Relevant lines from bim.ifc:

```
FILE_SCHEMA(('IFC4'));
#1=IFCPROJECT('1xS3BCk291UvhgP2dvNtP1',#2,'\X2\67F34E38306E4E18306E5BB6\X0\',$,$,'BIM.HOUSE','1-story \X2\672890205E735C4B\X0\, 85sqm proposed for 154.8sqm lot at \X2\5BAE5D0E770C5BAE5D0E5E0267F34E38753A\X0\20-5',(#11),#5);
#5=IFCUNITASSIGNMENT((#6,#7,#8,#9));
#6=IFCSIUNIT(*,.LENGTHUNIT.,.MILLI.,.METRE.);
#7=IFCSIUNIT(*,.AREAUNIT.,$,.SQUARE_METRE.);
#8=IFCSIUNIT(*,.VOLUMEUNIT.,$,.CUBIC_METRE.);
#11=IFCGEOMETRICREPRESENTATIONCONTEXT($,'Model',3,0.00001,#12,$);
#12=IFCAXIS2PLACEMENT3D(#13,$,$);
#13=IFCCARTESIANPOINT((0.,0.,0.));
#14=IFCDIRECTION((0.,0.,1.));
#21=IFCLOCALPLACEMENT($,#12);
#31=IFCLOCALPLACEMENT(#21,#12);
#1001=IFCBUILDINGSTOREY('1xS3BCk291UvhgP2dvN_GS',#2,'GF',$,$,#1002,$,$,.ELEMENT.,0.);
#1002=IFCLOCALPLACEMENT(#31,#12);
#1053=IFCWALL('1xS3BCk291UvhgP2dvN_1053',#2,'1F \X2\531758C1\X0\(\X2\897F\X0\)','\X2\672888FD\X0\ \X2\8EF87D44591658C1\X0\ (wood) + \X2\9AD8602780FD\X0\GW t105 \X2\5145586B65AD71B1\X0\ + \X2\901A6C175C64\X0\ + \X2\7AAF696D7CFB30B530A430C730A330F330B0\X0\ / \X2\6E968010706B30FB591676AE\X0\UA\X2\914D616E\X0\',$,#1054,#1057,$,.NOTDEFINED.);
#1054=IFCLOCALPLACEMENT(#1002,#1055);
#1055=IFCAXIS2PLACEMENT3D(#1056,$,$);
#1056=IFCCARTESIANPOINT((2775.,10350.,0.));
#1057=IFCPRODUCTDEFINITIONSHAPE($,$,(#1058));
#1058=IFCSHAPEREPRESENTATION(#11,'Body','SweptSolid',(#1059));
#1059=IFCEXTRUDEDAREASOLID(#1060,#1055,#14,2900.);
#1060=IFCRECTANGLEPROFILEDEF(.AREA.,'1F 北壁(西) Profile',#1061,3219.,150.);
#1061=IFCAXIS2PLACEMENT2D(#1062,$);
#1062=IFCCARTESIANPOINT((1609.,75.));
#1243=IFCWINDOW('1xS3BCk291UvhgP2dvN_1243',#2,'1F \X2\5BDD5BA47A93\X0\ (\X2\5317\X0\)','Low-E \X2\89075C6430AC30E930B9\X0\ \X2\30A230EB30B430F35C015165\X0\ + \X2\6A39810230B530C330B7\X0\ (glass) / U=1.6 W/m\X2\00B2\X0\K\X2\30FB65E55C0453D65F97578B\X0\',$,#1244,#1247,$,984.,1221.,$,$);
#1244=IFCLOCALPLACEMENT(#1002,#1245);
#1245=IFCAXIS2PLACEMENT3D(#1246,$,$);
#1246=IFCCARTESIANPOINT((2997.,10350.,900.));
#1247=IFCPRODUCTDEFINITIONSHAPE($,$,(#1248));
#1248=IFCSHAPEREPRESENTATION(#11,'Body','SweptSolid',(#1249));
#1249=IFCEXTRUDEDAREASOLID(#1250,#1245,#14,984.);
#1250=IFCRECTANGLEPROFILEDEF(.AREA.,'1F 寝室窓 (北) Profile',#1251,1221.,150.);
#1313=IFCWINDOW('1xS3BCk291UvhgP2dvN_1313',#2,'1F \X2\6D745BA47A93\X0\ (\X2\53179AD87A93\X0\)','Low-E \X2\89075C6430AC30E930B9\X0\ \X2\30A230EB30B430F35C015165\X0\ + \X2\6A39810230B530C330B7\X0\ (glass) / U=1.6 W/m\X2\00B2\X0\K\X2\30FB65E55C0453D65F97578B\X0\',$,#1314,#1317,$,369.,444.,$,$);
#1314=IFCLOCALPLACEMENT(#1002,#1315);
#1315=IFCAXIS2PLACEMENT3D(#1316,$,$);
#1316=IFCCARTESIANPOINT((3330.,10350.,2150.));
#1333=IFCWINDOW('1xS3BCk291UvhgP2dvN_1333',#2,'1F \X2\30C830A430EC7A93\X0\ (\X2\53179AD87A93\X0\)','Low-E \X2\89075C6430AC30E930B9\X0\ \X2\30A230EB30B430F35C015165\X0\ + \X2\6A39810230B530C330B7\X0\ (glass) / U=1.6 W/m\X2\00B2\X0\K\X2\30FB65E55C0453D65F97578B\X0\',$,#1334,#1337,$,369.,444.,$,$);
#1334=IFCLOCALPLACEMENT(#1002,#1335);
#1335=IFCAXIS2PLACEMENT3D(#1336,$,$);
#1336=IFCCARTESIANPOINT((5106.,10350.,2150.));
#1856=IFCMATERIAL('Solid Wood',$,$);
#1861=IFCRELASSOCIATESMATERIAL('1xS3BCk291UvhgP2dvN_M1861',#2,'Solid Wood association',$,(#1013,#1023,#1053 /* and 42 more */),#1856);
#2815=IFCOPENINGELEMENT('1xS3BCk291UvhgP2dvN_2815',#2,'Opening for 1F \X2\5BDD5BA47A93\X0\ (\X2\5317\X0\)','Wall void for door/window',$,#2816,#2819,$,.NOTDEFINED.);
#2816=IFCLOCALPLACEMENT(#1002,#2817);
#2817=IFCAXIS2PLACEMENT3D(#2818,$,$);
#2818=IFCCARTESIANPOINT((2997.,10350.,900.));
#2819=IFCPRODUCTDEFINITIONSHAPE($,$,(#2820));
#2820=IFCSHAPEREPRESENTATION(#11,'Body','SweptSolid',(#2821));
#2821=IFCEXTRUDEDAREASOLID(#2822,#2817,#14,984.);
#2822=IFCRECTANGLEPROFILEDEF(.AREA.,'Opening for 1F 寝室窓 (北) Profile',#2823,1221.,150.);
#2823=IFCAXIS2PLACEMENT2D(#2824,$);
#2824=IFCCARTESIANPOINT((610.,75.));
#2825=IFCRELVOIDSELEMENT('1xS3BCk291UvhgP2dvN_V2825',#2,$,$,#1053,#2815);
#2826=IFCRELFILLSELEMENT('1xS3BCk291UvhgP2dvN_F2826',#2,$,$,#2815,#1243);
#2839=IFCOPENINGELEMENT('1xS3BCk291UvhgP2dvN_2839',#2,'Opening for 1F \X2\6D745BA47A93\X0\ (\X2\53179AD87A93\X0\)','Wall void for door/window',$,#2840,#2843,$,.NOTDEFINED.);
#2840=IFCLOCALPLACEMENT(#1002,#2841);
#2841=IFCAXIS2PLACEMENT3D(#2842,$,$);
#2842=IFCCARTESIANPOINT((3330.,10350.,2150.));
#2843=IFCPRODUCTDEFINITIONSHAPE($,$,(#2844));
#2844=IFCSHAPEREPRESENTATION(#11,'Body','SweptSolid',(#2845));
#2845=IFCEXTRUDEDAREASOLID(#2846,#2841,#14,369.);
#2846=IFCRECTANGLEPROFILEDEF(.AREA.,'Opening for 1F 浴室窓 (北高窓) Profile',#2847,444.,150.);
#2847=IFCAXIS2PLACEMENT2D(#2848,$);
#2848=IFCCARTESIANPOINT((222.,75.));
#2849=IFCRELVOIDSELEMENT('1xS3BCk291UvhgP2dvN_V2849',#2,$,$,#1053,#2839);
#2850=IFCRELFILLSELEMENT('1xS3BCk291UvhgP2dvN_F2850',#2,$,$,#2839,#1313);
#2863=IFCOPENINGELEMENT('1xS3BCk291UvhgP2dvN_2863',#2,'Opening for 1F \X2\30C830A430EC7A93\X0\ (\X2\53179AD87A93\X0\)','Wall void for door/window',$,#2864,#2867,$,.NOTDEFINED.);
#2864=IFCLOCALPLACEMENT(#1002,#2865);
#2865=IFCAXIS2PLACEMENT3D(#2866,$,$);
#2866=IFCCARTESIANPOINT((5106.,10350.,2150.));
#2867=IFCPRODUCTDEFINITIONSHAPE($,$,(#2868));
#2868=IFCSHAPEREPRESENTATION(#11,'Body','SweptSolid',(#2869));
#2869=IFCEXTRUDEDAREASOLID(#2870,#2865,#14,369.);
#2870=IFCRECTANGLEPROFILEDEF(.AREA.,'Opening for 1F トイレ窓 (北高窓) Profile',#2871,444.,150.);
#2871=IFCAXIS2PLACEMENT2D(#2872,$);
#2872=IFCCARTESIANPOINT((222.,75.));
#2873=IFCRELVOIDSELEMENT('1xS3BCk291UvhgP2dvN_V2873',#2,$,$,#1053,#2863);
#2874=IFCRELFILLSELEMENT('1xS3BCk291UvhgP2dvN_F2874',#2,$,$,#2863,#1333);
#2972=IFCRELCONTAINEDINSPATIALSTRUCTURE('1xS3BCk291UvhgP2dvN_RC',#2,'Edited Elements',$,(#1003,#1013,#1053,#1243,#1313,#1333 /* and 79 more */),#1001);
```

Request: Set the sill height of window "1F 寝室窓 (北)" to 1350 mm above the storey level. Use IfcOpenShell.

```python
import numpy as np
import ifcopenshell
import ifcopenshell.api.geometry
import ifcopenshell.geom
import ifcopenshell.util.element
import ifcopenshell.util.placement
import ifcopenshell.util.shape
import ifcopenshell.util.unit

model = ifcopenshell.open("bim.ifc")
unit_scale = ifcopenshell.util.unit.calculate_unit_scale(model)

window = model.by_id(1243)
opening = window.FillsVoids[0].RelatingOpeningElement
storey = ifcopenshell.util.element.get_container(window, ifc_class="IfcBuildingStorey")
level = ifcopenshell.util.placement.get_local_placement(storey.ObjectPlacement)[2, 3]

# The opening's origin need not be at the sill, so measure its lowest point.
shape = ifcopenshell.geom.create_shape(ifcopenshell.geom.settings(), opening)
bottom = ifcopenshell.util.shape.get_shape_bottom_elevation(shape, shape.geometry) / unit_scale
dz = level + 1350.0 - bottom

shift = np.array([0.0, 0.0, dz])
# The window is not placed relative to its opening, so move both.
for product in (opening, window):
    matrix = ifcopenshell.util.placement.get_local_placement(product.ObjectPlacement)
    matrix[:3, 3] += shift
    ifcopenshell.api.geometry.edit_object_placement(model, product=product, matrix=matrix, is_si=False)

print(f"moved by {dz * unit_scale:+.3f} m")

model.write("bim-out.ifc")
```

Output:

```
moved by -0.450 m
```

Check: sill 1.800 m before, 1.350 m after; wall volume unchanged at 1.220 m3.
